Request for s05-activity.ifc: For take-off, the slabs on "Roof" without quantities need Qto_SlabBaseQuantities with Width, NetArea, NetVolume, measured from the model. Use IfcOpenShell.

First a look at what the model holds.

```python
import ifcopenshell
import ifcopenshell.util.element
import ifcopenshell.util.unit

model = ifcopenshell.open("s05-activity.ifc")
print(model.schema)
for unit_type in ("LENGTHUNIT", "AREAUNIT", "VOLUMEUNIT"):
    print(unit_type, ifcopenshell.util.unit.calculate_unit_scale(model, unit_type))
storey = next(s for s in model.by_type("IfcBuildingStorey") if s.Name == "Roof")
slabs = [e for e in ifcopenshell.util.element.get_decomposition(storey) if e.is_a("IfcSlab")]
for e in sorted(slabs, key=lambda e: e.id()):
    print(e.id(), e.is_a(), e.Name, list(ifcopenshell.util.element.get_psets(e, qtos_only=True)), sep=" | ")
```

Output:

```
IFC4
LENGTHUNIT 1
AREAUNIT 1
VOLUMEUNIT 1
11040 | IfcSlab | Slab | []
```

```python
import ifcopenshell
import ifcopenshell.api.pset
import ifcopenshell.geom
import ifcopenshell.util.element
import ifcopenshell.util.shape
import ifcopenshell.util.unit

model = ifcopenshell.open("s05-activity.ifc")
unit_scale = ifcopenshell.util.unit.calculate_unit_scale(model)
area_scale = ifcopenshell.util.unit.calculate_unit_scale(model, "AREAUNIT")
volume_scale = ifcopenshell.util.unit.calculate_unit_scale(model, "VOLUMEUNIT")
settings = ifcopenshell.geom.settings()

storey = next(s for s in model.by_type("IfcBuildingStorey") if s.Name == "Roof")
slabs = [e for e in ifcopenshell.util.element.get_decomposition(storey) if e.is_a("IfcSlab")]

for e in sorted(slabs, key=lambda e: e.id()):
    if ifcopenshell.util.element.get_psets(e, qtos_only=True, should_inherit=False):
        continue
    # Geometry comes back in metres, in the element's own axes.
    shape = ifcopenshell.geom.create_shape(settings, e)
    values = {
        "Width": ifcopenshell.util.shape.get_z(shape.geometry) / unit_scale,
        "NetArea": ifcopenshell.util.shape.get_footprint_area(shape.geometry) / area_scale,
        "NetVolume": ifcopenshell.util.shape.get_volume(shape.geometry) / volume_scale,
    }
    qto = ifcopenshell.api.pset.add_qto(model, product=e, name="Qto_SlabBaseQuantities")
    ifcopenshell.api.pset.edit_qto(model, qto=qto, properties=values)
    print(e.id(), {k: round(v, 3) for k, v in values.items()})

model.write("s05-activity-out.ifc")
```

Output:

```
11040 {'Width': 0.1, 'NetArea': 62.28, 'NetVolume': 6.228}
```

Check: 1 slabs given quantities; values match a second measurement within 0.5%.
